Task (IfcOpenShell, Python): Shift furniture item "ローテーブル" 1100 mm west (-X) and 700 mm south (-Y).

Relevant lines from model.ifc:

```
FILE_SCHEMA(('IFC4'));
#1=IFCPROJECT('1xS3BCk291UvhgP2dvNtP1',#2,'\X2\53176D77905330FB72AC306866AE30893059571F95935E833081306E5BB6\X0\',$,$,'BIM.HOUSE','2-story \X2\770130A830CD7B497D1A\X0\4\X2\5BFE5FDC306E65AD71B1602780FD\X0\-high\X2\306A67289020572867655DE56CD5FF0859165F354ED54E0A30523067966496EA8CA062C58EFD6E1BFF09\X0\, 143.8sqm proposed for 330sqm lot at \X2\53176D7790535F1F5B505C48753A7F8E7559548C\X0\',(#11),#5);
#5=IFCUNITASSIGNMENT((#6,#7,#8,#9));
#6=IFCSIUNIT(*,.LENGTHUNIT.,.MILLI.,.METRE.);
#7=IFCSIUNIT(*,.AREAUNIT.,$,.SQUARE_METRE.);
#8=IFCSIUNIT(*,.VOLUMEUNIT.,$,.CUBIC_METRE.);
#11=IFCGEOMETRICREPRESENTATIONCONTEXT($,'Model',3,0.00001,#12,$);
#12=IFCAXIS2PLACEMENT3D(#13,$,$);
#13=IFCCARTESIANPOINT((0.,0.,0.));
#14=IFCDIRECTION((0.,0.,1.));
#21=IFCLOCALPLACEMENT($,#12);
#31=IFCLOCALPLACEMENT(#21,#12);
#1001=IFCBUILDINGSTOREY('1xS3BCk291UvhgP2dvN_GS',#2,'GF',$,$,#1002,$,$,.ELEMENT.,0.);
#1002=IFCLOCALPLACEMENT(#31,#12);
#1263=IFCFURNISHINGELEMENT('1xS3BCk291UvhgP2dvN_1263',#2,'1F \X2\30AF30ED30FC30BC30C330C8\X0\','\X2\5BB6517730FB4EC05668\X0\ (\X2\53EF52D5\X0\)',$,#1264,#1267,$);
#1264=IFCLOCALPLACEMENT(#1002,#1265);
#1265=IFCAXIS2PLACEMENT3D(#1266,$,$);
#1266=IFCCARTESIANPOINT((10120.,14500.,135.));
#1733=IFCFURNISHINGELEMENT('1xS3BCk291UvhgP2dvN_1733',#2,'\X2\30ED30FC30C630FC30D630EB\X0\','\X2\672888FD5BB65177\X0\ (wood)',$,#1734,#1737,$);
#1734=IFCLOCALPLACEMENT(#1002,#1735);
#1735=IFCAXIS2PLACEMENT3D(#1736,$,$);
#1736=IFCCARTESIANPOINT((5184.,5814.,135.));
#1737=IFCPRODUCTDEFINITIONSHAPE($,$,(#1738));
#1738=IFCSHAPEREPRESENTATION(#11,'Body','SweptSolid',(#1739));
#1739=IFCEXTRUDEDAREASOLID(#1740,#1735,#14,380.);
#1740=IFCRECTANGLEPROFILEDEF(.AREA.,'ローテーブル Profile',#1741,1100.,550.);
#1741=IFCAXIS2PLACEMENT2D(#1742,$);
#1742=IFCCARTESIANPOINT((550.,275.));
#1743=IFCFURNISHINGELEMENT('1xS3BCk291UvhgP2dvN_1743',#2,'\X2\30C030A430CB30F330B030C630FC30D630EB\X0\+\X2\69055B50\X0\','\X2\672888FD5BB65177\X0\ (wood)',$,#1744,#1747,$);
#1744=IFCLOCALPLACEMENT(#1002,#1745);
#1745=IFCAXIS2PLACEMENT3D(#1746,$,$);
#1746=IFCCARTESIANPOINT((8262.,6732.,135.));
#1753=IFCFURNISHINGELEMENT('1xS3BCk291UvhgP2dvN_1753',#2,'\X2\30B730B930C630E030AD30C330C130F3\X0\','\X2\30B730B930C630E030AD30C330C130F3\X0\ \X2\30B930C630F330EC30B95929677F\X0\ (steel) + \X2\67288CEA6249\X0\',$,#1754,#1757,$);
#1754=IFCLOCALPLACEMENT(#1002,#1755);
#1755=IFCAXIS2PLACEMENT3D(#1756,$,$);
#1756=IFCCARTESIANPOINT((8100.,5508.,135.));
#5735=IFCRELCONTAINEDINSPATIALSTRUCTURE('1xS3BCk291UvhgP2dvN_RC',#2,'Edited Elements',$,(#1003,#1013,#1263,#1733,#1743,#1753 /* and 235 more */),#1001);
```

```python
import ifcopenshell
import ifcopenshell.api.geometry
import ifcopenshell.util.placement
import ifcopenshell.util.unit

model = ifcopenshell.open("model.ifc")
unit_scale = ifcopenshell.util.unit.calculate_unit_scale(model)

item = model.by_guid("1xS3BCk291UvhgP2dvN_1733")
matrix = ifcopenshell.util.placement.get_local_placement(item.ObjectPlacement)
matrix[0, 3] -= 1.1 / unit_scale
matrix[1, 3] -= 0.7 / unit_scale
ifcopenshell.api.geometry.edit_object_placement(model, product=item, matrix=matrix, is_si=False)

print(ifcopenshell.util.placement.get_local_placement(item.ObjectPlacement).round(3) + 0.0)

model.write("model_edited.ifc")
```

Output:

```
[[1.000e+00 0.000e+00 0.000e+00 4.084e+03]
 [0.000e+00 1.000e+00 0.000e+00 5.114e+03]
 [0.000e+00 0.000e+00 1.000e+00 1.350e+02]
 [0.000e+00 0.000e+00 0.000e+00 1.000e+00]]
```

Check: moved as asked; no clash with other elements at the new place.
